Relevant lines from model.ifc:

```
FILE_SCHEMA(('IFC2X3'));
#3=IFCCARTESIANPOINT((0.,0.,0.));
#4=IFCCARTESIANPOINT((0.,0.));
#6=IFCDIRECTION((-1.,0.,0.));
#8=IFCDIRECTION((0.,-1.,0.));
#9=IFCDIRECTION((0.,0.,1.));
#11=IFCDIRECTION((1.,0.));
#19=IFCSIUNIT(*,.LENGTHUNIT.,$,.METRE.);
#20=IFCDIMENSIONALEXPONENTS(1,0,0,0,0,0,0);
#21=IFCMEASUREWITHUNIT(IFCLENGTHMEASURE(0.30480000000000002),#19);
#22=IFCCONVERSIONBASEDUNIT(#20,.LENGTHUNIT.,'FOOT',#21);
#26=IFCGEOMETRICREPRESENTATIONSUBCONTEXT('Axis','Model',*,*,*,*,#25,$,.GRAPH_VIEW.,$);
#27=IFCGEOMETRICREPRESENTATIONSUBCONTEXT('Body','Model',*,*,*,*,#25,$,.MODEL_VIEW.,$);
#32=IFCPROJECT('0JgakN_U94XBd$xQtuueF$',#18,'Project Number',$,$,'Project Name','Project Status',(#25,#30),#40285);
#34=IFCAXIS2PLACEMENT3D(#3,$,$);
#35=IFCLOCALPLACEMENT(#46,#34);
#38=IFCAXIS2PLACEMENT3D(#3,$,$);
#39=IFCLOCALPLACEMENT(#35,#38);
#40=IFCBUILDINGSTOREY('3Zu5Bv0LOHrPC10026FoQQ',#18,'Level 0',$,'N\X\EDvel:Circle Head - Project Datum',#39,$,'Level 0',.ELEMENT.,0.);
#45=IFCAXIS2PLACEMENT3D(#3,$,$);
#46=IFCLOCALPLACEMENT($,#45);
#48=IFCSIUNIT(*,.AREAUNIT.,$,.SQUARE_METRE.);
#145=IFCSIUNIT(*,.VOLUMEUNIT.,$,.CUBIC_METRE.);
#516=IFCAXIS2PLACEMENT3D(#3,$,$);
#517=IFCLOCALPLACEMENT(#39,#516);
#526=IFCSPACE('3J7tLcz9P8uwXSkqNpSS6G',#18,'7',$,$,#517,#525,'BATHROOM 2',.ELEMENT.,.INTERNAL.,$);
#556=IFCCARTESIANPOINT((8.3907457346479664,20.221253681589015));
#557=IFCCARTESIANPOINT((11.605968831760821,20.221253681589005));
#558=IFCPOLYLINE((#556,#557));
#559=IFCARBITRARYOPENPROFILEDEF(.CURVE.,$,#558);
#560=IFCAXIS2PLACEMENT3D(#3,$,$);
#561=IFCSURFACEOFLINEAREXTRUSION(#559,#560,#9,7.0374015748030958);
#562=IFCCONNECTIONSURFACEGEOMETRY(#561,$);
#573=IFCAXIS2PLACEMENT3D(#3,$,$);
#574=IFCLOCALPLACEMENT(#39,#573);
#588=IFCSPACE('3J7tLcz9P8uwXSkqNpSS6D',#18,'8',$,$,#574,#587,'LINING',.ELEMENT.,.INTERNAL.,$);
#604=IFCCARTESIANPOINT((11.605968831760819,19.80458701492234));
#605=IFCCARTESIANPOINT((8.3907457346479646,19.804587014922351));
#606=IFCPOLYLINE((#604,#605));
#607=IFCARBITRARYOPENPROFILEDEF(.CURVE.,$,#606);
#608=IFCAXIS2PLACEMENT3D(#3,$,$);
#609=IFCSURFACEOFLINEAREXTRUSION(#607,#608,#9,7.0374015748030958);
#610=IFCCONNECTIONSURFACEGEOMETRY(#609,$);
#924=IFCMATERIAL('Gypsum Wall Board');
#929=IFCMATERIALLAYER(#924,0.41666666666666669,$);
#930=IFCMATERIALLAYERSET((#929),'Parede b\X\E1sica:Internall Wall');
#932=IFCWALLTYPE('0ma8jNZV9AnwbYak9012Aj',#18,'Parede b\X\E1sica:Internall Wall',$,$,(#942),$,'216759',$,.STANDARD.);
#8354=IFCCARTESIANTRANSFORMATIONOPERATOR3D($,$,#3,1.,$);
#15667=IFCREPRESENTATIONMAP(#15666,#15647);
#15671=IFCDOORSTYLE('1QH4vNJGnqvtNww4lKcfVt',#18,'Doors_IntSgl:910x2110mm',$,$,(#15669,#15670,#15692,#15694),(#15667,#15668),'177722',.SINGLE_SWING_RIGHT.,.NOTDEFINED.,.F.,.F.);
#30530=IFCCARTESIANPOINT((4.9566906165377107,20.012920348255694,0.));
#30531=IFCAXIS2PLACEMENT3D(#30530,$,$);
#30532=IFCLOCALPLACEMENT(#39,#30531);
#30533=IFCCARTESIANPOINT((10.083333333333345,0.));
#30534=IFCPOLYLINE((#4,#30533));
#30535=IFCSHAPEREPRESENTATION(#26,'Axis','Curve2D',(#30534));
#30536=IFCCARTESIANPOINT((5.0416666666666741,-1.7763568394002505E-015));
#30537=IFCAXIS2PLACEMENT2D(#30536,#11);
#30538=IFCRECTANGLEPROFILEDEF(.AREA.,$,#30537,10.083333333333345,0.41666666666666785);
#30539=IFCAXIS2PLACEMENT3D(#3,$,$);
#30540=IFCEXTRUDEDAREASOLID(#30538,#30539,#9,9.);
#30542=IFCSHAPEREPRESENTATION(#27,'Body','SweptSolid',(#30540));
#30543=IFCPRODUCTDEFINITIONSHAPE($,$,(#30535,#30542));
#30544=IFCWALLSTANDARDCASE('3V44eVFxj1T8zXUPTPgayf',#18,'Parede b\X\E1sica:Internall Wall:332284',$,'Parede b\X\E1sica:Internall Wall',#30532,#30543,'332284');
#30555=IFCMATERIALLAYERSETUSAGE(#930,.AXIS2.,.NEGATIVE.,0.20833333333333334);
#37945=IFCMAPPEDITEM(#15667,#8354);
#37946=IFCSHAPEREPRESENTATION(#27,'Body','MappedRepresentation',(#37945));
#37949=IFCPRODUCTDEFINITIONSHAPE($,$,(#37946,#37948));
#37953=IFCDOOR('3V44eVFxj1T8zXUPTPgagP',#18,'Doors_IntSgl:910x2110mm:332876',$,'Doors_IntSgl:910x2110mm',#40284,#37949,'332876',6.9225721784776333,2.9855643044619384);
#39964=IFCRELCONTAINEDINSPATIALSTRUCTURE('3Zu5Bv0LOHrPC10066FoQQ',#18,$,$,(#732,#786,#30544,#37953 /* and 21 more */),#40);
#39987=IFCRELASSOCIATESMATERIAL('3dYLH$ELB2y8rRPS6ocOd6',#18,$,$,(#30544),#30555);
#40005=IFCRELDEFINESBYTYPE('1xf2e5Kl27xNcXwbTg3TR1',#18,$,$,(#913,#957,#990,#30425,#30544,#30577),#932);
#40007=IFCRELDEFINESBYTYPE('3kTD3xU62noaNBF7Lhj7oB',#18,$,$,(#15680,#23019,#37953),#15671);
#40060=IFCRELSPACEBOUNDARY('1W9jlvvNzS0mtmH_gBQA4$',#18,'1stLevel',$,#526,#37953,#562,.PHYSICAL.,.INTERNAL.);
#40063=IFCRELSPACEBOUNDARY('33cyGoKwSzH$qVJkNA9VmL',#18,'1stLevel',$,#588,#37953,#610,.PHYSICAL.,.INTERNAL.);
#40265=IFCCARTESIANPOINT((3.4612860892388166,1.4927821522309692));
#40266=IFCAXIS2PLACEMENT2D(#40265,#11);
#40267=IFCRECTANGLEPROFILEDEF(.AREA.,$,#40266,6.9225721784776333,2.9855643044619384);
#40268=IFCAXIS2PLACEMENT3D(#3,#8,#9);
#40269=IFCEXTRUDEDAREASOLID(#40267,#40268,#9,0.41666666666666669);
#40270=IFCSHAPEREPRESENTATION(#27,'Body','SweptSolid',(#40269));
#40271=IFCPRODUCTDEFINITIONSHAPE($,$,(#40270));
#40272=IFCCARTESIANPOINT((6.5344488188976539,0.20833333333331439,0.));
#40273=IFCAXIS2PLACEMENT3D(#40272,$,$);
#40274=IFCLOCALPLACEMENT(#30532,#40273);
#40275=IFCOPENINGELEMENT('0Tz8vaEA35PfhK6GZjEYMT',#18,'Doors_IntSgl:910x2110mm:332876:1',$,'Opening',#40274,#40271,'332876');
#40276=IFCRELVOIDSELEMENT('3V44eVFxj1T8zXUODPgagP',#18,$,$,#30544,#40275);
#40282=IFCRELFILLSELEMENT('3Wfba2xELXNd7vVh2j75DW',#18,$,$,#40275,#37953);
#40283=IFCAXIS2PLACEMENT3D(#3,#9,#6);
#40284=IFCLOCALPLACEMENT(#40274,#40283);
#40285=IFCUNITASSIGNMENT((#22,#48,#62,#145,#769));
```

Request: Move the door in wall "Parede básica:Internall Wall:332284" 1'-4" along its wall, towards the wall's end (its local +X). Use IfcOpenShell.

```python
import numpy as np
import ifcopenshell
import ifcopenshell.api.geometry
import ifcopenshell.util.placement
import ifcopenshell.util.unit

model = ifcopenshell.open("model.ifc")
unit_scale = ifcopenshell.util.unit.calculate_unit_scale(model)

door = model.by_guid("3V44eVFxj1T8zXUPTPgagP")
opening = door.FillsVoids[0].RelatingOpeningElement
wall = opening.VoidsElements[0].RelatingBuildingElement

wall_matrix = ifcopenshell.util.placement.get_local_placement(wall.ObjectPlacement)
shift = wall_matrix[:3, 0] * 16 * 0.0254 / unit_scale
before = ifcopenshell.util.placement.get_local_placement(door.ObjectPlacement)[:3, 3].copy()

# The door is placed relative to its opening, so it follows when the opening moves.
matrix = ifcopenshell.util.placement.get_local_placement(opening.ObjectPlacement)
matrix[:3, 3] += shift
ifcopenshell.api.geometry.edit_object_placement(
    model, product=opening, matrix=matrix, is_si=False, should_transform_children=True
)

# Space boundary surfaces are stored in each space's coordinates; move them too.
for rel in door.ProvidesBoundaries:
    if not rel.ConnectionGeometry:
        continue
    surface = rel.ConnectionGeometry.SurfaceOnRelatingElement
    space_matrix = ifcopenshell.util.placement.get_local_placement(rel.RelatingSpace.ObjectPlacement)
    point = np.array(surface.Position.Location.Coordinates) + space_matrix[:3, :3].T @ shift
    surface.Position = model.createIfcAxis2Placement3D(
        model.createIfcCartesianPoint(point.tolist()), surface.Position.Axis, surface.Position.RefDirection
    )

after = ifcopenshell.util.placement.get_local_placement(door.ObjectPlacement)[:3, 3]
print("door moved by", (after - before).round(3) + 0.0)

model.write("model_v2.ifc")
```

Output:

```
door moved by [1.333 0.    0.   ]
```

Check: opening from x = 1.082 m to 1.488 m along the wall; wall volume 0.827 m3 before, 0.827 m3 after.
